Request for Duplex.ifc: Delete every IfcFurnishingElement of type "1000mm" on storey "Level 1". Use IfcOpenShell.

First a look at what the model holds.

```python
import ifcopenshell
import ifcopenshell.util.element

model = ifcopenshell.open("Duplex.ifc")
print(model.schema)
storey = next(s for s in model.by_type("IfcBuildingStorey") if s.Name == "Level 1")
furniture = [e for e in ifcopenshell.util.element.get_decomposition(storey) if e.is_a("IfcFurnishingElement")]
seen = {}
for e in furniture:
    element_type = ifcopenshell.util.element.get_type(e)
    name = element_type.Name if element_type not in (None, e) else None
    seen[name] = seen.get(name, 0) + 1
for name, count in sorted(seen.items(), key=str):
    print(count, "x", name)
```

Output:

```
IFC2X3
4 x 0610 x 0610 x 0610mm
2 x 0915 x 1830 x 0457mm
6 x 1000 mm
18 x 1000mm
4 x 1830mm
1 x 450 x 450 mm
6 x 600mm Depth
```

```python
import ifcopenshell
import ifcopenshell.api.root
import ifcopenshell.util.element

model = ifcopenshell.open("Duplex.ifc")

storey = next(s for s in model.by_type("IfcBuildingStorey") if s.Name == "Level 1")
furniture = [e for e in ifcopenshell.util.element.get_decomposition(storey) if e.is_a("IfcFurnishingElement")]
targets = [e for e in furniture if (t := ifcopenshell.util.element.get_type(e)) not in (None, e) and t.Name == "1000mm"]

for e in targets:
    ifcopenshell.api.root.remove_product(model, product=e)
print(len(targets), "removed")

model.write("Duplex_rev.ifc")
```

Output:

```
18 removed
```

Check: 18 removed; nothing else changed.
